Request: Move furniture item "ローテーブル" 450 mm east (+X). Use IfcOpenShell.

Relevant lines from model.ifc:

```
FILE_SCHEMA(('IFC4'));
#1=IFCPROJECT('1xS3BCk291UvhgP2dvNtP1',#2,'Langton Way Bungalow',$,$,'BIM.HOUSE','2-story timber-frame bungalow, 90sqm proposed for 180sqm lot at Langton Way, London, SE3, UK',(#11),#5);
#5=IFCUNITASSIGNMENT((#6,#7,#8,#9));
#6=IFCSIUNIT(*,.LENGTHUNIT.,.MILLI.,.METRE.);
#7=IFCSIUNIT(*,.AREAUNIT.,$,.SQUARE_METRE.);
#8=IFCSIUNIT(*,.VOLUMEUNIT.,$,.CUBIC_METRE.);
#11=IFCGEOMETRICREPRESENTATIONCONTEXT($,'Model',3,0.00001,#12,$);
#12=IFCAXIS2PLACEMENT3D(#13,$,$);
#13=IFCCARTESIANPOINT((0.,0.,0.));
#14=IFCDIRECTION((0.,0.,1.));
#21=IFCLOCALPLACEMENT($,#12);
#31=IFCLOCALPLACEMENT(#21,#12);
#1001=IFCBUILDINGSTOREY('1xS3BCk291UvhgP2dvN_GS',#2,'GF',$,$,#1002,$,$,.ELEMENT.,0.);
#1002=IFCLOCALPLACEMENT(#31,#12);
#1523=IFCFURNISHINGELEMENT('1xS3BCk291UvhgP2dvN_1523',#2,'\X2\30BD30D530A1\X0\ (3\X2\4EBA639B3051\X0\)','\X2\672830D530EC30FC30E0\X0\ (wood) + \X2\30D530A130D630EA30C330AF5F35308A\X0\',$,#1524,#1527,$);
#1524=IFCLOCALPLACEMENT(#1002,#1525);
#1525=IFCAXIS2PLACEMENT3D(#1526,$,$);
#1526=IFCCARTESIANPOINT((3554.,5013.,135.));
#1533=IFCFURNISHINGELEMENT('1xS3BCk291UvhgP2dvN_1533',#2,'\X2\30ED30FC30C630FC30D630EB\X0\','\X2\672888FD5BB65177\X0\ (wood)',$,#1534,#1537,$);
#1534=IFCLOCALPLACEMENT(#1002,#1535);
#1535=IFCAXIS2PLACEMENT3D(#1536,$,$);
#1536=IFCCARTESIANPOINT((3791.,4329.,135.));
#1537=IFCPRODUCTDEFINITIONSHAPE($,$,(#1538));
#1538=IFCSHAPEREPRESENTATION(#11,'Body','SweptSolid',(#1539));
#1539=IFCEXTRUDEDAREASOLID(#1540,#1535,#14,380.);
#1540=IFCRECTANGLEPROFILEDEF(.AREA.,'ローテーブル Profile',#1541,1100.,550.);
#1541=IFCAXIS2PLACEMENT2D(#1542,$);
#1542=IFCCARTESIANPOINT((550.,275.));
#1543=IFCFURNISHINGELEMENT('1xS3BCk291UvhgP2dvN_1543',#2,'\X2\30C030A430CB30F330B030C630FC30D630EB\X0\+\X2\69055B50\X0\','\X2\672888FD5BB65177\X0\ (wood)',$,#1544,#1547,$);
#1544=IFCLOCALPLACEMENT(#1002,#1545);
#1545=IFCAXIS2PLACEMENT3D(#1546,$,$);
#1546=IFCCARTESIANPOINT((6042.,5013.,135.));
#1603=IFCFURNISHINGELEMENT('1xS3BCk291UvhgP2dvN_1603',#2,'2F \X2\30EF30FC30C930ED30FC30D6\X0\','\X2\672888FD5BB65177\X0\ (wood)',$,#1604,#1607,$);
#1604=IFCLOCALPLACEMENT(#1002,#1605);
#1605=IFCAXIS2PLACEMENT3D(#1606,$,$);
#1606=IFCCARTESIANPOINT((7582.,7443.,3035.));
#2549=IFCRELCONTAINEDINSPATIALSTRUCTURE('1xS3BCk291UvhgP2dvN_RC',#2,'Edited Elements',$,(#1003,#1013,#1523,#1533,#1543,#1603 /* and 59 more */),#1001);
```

```python
import ifcopenshell
import ifcopenshell.api.geometry
import ifcopenshell.util.placement

model = ifcopenshell.open("model.ifc")

item = model.by_guid("1xS3BCk291UvhgP2dvN_1533")
matrix = ifcopenshell.util.placement.get_local_placement(item.ObjectPlacement)
matrix[0, 3] += 450.0
ifcopenshell.api.geometry.edit_object_placement(model, product=item, matrix=matrix, is_si=False)

print(ifcopenshell.util.placement.get_local_placement(item.ObjectPlacement).round(3) + 0.0)

model.write("model_rev.ifc")
```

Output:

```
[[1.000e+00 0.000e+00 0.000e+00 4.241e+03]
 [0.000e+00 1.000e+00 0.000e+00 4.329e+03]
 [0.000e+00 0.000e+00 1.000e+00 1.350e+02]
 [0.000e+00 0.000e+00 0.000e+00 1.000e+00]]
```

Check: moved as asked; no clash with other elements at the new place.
